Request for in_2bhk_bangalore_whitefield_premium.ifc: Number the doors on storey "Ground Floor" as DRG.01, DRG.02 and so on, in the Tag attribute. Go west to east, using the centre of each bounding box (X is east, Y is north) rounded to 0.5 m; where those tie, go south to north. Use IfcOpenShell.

First a look at what the model holds.

```python
import ifcopenshell
import ifcopenshell.util.element
import ifcopenshell.util.placement

model = ifcopenshell.open("in_2bhk_bangalore_whitefield_premium.ifc")
print(model.schema)
storey = next(s for s in model.by_type("IfcBuildingStorey") if s.Name == "Ground Floor")
doors = [e for e in ifcopenshell.util.element.get_decomposition(storey) if e.is_a("IfcDoor")]
for e in sorted(doors, key=lambda e: e.id()):
    origin = ifcopenshell.util.placement.get_local_placement(e.ObjectPlacement)[:3, 3]
    print(e.id(), e.Tag, e.Name, origin.round(2) + 0.0, sep=" | ")
```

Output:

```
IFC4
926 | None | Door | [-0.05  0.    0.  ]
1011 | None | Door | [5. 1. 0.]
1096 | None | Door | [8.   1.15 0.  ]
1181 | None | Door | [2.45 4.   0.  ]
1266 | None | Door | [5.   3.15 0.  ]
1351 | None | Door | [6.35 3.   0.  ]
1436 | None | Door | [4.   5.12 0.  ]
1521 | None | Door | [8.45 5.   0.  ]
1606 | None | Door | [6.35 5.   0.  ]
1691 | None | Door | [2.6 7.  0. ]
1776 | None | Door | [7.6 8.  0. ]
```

```python
import ifcopenshell
import ifcopenshell.geom
import ifcopenshell.util.element
import ifcopenshell.util.shape

model = ifcopenshell.open("in_2bhk_bangalore_whitefield_premium.ifc")
settings = ifcopenshell.geom.settings()
settings.set("use-world-coords", True)


def centre(element):
    shape = ifcopenshell.geom.create_shape(settings, element)
    return ifcopenshell.util.shape.get_bbox_centroid(shape.geometry)


storey = next(s for s in model.by_type("IfcBuildingStorey") if s.Name == "Ground Floor")
doors = [e for e in ifcopenshell.util.element.get_decomposition(storey) if e.is_a("IfcDoor")]

# Insertion points can sit at a corner or the storey origin, so sort by the geometry (in metres).
centres = {e: centre(e) for e in doors}
doors.sort(key=lambda e: (round(centres[e][0] / 0.5), centres[e][1]))

for i, e in enumerate(doors, start=1):
    number = f"DRG.{i:02d}"
    e.Tag = number
    print(e.id(), number)

model.write("in_2bhk_bangalore_whitefield_premium_updated.ifc")
```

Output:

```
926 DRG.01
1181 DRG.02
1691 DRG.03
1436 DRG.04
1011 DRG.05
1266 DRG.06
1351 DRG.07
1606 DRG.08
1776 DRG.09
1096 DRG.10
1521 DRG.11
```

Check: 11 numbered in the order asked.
